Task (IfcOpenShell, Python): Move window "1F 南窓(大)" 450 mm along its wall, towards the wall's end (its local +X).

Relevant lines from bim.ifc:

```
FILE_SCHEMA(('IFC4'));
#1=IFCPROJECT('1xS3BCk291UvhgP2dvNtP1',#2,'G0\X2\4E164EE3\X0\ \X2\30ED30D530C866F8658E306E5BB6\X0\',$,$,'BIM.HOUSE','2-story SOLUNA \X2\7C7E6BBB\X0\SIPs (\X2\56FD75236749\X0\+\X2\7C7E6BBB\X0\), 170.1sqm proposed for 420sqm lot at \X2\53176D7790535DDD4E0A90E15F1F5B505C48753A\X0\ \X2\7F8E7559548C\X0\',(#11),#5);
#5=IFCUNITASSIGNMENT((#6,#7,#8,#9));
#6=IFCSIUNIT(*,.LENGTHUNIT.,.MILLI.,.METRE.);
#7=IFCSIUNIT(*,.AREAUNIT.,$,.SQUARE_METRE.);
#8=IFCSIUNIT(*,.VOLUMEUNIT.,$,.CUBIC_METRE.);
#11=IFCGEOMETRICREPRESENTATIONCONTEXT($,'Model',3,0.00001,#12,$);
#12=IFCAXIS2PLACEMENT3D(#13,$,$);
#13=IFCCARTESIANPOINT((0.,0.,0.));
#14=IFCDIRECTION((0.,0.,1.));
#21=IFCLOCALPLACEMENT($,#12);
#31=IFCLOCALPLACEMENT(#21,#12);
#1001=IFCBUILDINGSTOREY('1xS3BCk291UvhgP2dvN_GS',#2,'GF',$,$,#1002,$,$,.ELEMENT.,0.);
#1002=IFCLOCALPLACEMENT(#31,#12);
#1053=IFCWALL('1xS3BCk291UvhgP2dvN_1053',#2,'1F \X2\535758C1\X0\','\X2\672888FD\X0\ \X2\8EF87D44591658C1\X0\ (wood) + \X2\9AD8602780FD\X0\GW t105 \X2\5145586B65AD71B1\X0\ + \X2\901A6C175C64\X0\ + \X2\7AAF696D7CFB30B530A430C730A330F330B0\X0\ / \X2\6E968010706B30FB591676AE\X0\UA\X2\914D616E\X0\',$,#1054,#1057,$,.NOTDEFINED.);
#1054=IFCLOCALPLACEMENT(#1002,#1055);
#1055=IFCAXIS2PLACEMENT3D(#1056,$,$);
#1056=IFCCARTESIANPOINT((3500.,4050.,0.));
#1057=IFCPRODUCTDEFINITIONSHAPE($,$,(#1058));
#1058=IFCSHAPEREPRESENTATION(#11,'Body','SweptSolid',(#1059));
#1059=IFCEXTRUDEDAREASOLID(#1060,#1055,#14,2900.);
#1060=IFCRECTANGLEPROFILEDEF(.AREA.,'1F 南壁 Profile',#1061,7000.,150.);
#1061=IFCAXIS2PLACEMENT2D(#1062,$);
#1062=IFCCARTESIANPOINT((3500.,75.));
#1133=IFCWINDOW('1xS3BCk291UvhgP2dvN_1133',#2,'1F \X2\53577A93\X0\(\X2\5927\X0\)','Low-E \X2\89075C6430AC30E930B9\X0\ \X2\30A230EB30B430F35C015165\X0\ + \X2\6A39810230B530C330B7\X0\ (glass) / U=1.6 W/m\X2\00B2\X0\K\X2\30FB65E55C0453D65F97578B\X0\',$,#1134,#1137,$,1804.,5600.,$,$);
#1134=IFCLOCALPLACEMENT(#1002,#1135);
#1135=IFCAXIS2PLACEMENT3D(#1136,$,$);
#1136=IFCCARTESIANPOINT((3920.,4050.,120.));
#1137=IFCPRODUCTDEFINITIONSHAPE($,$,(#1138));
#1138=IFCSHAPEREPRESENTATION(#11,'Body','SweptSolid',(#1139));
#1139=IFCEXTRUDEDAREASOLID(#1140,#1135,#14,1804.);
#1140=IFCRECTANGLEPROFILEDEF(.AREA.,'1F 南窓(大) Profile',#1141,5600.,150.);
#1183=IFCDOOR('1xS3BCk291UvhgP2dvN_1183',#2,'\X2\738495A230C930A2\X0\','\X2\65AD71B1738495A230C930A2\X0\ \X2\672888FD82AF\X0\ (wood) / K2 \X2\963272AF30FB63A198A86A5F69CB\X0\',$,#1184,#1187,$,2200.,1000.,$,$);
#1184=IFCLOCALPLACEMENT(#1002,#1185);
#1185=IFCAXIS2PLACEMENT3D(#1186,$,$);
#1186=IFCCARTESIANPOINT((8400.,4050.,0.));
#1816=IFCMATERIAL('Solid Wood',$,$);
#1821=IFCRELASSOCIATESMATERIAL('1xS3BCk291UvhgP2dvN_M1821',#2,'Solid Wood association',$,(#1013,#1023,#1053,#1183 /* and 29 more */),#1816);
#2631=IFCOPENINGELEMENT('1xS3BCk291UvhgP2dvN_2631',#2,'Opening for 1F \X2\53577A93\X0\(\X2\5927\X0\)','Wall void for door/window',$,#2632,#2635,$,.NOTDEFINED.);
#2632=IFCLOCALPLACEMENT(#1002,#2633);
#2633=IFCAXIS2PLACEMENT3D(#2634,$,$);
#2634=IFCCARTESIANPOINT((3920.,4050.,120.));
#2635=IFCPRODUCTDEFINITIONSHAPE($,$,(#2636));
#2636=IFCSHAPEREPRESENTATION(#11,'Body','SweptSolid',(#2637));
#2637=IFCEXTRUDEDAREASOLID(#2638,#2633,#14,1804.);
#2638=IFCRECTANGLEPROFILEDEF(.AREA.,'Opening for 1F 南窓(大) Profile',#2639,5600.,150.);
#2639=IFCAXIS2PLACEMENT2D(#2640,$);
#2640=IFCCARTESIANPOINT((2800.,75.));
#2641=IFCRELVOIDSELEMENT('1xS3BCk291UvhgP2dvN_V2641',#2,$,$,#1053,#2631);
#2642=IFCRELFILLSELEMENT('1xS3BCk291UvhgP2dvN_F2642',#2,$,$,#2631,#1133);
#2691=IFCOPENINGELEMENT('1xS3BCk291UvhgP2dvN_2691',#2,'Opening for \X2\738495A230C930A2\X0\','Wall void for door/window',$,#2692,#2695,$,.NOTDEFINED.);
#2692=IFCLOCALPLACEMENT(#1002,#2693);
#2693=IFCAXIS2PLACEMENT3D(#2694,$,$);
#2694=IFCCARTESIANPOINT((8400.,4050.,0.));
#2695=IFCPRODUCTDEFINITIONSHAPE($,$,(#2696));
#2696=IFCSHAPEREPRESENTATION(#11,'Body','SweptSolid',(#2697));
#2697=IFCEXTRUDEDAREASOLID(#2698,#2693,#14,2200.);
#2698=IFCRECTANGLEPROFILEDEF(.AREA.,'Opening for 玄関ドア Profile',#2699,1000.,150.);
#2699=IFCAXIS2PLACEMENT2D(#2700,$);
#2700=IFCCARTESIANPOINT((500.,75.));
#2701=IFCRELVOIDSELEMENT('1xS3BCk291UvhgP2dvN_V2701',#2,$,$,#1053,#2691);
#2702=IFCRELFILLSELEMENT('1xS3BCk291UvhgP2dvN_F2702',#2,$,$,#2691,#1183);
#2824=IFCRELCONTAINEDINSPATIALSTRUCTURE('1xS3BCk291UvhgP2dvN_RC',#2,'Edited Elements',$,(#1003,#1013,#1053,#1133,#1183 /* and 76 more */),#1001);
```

```python
import ifcopenshell
import ifcopenshell.api.geometry
import ifcopenshell.util.placement

model = ifcopenshell.open("bim.ifc")

window = model.by_guid("1xS3BCk291UvhgP2dvN_1133")
opening = window.FillsVoids[0].RelatingOpeningElement
wall = opening.VoidsElements[0].RelatingBuildingElement

wall_matrix = ifcopenshell.util.placement.get_local_placement(wall.ObjectPlacement)
shift = wall_matrix[:3, 0] * 450.0
before = ifcopenshell.util.placement.get_local_placement(window.ObjectPlacement)[:3, 3].copy()

# The window is not placed relative to its opening, so move both.
for product in (opening, window):
    matrix = ifcopenshell.util.placement.get_local_placement(product.ObjectPlacement)
    matrix[:3, 3] += shift
    ifcopenshell.api.geometry.edit_object_placement(model, product=product, matrix=matrix, is_si=False)

after = ifcopenshell.util.placement.get_local_placement(window.ObjectPlacement)[:3, 3]
print("window moved by", (after - before).round(3) + 0.0)

model.write("bim_v2.ifc")
```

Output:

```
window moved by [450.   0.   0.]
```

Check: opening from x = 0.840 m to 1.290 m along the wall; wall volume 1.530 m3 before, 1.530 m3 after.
